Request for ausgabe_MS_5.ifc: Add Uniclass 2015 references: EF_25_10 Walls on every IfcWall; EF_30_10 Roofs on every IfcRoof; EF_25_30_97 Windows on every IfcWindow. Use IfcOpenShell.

First a look at what the model holds.

```python
import ifcopenshell

model = ifcopenshell.open("ausgabe_MS_5.ifc")
print(model.schema)
print("classifications:", [c.Name for c in model.by_type("IfcClassification")])
for ifc_class in ("IfcDoor", "IfcRoof", "IfcStair", "IfcWall", "IfcWindow"):
    print(ifc_class, len(model.by_type(ifc_class)))
```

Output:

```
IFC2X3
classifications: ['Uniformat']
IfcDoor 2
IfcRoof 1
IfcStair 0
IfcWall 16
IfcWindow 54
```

```python
import ifcopenshell
import ifcopenshell.api.classification

model = ifcopenshell.open("ausgabe_MS_5.ifc")

# IFC2X3 requires Source and Edition and has no link from the project to the system.
system = model.create_entity("IfcClassification", Source="NBS", Edition="2015", Name="Uniclass 2015")

codes = {
    "IfcWall": ("EF_25_10", "Walls"),
    "IfcRoof": ("EF_30_10", "Roofs"),
    "IfcWindow": ("EF_25_30_97", "Windows"),
}
for ifc_class, (code, name) in codes.items():
    products = model.by_type(ifc_class)
    ifcopenshell.api.classification.add_reference(
        model, products=products, classification=system, identification=code, name=name
    )
    print(code, len(products))

model.write("ausgabe_MS_5_v2.ifc")
```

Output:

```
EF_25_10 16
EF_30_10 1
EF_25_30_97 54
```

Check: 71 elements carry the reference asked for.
